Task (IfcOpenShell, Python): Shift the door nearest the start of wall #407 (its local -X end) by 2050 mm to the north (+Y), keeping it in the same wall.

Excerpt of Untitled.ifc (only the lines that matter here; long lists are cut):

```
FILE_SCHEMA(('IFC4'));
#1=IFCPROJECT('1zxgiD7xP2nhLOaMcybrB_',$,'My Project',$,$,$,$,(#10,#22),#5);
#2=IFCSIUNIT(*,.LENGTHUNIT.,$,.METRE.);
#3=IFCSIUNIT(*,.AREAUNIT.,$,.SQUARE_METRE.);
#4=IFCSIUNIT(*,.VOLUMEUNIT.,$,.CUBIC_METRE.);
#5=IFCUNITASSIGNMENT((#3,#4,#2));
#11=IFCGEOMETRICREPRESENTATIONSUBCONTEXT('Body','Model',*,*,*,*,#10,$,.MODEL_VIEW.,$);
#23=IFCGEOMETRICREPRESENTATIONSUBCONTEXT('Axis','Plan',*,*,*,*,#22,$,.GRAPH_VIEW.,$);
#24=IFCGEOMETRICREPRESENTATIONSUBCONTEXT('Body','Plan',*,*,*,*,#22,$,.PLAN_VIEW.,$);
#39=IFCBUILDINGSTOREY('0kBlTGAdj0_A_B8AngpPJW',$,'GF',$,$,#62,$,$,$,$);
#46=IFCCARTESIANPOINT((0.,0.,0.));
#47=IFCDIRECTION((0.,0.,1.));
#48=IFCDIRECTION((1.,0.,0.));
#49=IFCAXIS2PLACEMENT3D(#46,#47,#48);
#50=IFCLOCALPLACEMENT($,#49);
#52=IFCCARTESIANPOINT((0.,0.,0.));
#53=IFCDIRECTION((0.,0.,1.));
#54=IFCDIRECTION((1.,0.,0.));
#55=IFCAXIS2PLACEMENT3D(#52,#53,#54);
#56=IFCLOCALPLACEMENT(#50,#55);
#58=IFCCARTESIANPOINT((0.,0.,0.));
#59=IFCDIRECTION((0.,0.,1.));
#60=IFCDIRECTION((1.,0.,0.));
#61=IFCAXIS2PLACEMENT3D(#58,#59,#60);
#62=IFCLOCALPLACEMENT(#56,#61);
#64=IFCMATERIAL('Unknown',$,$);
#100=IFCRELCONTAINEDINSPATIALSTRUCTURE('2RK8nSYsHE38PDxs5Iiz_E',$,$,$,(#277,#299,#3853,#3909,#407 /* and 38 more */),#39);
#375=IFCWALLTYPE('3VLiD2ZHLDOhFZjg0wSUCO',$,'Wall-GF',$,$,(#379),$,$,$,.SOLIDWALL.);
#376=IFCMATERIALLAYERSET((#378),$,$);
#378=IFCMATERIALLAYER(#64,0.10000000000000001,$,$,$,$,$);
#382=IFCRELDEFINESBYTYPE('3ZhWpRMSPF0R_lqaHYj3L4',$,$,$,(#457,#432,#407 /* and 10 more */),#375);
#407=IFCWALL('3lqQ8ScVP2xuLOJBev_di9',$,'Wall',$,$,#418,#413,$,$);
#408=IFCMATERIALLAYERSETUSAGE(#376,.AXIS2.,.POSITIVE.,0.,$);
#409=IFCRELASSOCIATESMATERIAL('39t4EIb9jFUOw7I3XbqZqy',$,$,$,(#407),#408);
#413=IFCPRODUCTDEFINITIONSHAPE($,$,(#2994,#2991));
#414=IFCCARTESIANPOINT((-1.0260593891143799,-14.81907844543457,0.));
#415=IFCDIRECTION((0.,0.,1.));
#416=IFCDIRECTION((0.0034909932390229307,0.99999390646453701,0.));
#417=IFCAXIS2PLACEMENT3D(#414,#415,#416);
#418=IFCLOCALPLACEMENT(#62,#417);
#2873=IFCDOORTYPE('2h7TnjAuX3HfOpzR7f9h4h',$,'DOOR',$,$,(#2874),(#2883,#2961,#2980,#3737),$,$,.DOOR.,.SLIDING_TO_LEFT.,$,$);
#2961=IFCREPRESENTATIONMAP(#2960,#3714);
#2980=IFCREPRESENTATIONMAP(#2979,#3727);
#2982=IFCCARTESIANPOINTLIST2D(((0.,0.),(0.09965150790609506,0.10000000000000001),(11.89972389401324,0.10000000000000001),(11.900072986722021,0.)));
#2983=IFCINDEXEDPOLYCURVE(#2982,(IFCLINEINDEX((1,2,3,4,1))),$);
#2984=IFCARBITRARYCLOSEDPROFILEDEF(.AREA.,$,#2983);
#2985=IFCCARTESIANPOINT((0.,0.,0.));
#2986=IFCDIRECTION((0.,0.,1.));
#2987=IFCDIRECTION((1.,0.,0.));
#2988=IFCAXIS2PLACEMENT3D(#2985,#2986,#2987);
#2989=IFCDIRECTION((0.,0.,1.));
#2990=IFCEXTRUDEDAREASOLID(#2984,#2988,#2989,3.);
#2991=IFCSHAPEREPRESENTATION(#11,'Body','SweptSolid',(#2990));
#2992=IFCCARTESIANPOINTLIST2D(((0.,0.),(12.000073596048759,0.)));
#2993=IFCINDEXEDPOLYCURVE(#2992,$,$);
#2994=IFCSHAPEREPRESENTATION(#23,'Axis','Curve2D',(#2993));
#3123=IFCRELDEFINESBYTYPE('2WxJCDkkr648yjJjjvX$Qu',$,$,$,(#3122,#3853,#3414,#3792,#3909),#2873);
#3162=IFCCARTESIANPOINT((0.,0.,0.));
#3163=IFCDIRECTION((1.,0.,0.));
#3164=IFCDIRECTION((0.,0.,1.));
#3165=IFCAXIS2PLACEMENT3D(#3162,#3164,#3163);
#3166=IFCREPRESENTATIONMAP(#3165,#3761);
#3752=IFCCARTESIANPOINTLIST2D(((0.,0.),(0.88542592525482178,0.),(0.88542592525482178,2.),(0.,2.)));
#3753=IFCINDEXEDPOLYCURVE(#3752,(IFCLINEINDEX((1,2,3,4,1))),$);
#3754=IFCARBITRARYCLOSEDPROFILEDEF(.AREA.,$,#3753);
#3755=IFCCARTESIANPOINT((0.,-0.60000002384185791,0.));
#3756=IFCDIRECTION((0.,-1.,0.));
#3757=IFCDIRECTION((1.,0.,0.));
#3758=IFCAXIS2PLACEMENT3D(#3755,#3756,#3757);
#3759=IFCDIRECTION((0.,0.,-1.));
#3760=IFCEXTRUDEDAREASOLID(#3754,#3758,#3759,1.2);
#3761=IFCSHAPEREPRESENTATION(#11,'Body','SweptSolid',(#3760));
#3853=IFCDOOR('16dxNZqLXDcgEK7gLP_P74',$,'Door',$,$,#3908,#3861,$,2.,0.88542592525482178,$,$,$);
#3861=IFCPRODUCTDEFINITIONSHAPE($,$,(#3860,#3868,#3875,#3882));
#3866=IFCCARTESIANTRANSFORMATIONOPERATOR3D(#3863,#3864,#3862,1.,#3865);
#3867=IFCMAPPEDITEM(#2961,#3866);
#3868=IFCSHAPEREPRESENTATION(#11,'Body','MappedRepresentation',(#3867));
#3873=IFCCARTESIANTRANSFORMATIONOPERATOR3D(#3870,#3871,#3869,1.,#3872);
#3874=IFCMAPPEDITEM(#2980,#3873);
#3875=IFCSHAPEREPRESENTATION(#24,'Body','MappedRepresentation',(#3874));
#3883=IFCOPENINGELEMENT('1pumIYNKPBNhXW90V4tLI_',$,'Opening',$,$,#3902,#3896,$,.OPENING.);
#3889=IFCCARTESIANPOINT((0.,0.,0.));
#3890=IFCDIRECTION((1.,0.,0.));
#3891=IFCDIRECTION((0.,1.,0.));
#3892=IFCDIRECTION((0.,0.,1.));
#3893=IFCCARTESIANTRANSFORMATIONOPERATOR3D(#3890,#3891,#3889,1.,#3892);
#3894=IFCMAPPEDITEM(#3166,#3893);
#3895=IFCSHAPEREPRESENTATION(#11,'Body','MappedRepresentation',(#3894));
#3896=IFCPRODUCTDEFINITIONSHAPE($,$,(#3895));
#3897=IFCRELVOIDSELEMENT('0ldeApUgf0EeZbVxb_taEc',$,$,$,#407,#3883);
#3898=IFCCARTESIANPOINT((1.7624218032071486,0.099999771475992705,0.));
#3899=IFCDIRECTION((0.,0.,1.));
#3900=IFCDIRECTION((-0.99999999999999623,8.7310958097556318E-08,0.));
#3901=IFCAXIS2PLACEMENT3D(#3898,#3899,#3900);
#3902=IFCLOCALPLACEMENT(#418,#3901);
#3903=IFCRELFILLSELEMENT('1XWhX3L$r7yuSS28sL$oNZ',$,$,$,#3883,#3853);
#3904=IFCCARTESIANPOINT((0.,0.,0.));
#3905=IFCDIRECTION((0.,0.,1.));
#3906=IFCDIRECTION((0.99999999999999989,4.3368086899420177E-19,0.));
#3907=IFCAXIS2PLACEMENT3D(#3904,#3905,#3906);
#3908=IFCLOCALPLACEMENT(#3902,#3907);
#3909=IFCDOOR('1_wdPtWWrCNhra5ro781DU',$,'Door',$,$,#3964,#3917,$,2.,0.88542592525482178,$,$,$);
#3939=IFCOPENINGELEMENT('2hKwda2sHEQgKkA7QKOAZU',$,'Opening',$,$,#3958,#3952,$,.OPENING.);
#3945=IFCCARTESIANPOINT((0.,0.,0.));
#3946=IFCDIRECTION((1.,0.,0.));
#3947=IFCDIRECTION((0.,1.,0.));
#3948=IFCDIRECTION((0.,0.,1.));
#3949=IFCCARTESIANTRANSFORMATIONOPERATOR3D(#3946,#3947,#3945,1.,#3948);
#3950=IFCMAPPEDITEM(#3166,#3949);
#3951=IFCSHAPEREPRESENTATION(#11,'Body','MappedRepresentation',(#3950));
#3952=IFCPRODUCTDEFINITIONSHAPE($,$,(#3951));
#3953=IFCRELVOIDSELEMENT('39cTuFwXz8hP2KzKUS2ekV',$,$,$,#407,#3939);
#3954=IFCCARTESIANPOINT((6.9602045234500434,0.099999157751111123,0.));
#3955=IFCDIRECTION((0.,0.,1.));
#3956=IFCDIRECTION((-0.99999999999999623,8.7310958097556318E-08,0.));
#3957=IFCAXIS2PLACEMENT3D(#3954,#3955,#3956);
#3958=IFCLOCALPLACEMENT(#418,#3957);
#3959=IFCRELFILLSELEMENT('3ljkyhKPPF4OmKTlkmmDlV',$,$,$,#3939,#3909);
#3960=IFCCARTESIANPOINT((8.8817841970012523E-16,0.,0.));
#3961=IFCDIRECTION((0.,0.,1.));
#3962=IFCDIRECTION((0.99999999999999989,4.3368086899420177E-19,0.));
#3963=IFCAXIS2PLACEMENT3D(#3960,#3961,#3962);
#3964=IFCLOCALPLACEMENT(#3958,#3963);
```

```python
import ifcopenshell
import ifcopenshell.api.geometry
import ifcopenshell.util.placement

model = ifcopenshell.open("Untitled.ifc")

door = model.by_guid("16dxNZqLXDcgEK7gLP_P74")
opening = door.FillsVoids[0].RelatingOpeningElement
wall = opening.VoidsElements[0].RelatingBuildingElement

wall_matrix = ifcopenshell.util.placement.get_local_placement(wall.ObjectPlacement)
shift = wall_matrix[:3, 0] * 2.05
before = ifcopenshell.util.placement.get_local_placement(door.ObjectPlacement)[:3, 3].copy()

# The door is placed relative to its opening, so it follows when the opening moves.
matrix = ifcopenshell.util.placement.get_local_placement(opening.ObjectPlacement)
matrix[:3, 3] += shift
ifcopenshell.api.geometry.edit_object_placement(
    model, product=opening, matrix=matrix, is_si=False, should_transform_children=True
)

after = ifcopenshell.util.placement.get_local_placement(door.ObjectPlacement)[:3, 3]
print("door moved by", (after - before).round(3) + 0.0)

model.write("Untitled_v2.ifc")
```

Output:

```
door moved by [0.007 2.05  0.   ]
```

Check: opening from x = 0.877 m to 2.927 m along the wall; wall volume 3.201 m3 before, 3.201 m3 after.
